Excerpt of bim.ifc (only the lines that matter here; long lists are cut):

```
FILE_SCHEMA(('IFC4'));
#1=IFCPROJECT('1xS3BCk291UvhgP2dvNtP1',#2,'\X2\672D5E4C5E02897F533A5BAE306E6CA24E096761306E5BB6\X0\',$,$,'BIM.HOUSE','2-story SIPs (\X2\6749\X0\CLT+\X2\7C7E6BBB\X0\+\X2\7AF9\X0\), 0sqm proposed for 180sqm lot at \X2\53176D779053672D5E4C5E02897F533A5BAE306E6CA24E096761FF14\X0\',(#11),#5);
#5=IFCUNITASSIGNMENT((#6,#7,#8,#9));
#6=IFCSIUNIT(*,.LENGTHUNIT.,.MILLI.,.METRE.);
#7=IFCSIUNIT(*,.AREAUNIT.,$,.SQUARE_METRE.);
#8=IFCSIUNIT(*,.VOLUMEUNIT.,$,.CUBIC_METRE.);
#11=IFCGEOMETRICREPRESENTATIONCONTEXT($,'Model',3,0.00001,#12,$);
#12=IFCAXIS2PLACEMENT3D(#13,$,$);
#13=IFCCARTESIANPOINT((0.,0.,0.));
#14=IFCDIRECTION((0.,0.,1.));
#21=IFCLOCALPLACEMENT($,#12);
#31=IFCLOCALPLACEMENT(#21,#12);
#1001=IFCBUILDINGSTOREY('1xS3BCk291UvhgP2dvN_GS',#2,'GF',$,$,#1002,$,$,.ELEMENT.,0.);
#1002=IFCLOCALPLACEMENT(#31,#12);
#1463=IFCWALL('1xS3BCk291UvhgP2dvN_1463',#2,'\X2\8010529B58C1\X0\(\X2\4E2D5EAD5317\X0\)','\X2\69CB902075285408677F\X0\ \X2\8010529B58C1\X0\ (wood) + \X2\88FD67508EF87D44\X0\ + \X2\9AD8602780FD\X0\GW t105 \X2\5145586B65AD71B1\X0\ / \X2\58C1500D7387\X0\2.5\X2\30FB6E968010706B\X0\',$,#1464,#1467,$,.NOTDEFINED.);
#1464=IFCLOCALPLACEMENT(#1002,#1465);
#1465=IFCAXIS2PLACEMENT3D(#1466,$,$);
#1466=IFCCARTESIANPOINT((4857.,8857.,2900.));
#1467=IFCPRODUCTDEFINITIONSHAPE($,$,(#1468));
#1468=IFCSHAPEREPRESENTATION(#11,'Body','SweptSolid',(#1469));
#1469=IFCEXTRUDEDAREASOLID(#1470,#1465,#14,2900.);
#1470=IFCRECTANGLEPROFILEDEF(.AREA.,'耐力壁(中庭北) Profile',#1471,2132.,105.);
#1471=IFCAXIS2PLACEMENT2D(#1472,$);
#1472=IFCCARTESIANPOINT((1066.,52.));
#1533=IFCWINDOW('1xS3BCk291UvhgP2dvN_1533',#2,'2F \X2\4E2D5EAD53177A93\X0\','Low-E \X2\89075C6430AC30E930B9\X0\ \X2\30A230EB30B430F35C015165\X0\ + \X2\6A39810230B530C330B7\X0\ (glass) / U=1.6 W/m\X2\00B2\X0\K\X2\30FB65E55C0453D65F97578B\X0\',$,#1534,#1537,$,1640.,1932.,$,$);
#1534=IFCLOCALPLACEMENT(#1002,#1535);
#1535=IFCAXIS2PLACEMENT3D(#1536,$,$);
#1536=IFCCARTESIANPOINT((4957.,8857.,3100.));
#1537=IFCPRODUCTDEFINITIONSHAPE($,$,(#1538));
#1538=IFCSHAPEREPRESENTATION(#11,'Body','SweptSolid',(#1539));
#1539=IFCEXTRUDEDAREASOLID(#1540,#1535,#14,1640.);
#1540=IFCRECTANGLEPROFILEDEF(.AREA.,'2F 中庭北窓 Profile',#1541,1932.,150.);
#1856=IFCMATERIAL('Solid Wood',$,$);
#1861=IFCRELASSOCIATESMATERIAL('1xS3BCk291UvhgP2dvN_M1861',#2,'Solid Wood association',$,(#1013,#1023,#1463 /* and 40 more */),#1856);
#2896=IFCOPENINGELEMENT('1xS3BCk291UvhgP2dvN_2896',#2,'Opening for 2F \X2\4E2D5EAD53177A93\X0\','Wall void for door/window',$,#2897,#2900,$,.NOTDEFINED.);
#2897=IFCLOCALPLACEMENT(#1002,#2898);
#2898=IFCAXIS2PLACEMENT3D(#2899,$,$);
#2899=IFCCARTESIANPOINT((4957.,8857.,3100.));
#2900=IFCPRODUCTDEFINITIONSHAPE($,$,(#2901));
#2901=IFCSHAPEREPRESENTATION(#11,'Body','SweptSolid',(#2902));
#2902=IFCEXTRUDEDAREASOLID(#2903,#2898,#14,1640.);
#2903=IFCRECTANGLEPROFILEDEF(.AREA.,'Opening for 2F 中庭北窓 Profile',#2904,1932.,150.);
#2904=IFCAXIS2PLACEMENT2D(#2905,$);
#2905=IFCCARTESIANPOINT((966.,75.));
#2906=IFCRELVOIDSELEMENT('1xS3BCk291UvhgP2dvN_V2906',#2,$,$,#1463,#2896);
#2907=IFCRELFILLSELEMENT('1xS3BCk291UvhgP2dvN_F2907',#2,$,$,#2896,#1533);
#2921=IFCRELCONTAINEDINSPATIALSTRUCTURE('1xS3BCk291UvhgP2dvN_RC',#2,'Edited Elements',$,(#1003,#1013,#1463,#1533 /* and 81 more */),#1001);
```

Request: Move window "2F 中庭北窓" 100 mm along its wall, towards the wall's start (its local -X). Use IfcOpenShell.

```python
import ifcopenshell
import ifcopenshell.api.geometry
import ifcopenshell.util.placement
import ifcopenshell.util.unit

model = ifcopenshell.open("bim.ifc")
unit_scale = ifcopenshell.util.unit.calculate_unit_scale(model)

window = model.by_guid("1xS3BCk291UvhgP2dvN_1533")
opening = window.FillsVoids[0].RelatingOpeningElement
wall = opening.VoidsElements[0].RelatingBuildingElement

wall_matrix = ifcopenshell.util.placement.get_local_placement(wall.ObjectPlacement)
shift = wall_matrix[:3, 0] * -0.1 / unit_scale
before = ifcopenshell.util.placement.get_local_placement(window.ObjectPlacement)[:3, 3].copy()

# The window is not placed relative to its opening, so move both.
for product in (opening, window):
    matrix = ifcopenshell.util.placement.get_local_placement(product.ObjectPlacement)
    matrix[:3, 3] += shift
    ifcopenshell.api.geometry.edit_object_placement(model, product=product, matrix=matrix, is_si=False)

after = ifcopenshell.util.placement.get_local_placement(window.ObjectPlacement)[:3, 3]
print("window moved by", (after - before).round(3) + 0.0)

model.write("bim_v2.ifc")
```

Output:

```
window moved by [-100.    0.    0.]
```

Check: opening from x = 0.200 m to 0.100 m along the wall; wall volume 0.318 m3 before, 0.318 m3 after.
